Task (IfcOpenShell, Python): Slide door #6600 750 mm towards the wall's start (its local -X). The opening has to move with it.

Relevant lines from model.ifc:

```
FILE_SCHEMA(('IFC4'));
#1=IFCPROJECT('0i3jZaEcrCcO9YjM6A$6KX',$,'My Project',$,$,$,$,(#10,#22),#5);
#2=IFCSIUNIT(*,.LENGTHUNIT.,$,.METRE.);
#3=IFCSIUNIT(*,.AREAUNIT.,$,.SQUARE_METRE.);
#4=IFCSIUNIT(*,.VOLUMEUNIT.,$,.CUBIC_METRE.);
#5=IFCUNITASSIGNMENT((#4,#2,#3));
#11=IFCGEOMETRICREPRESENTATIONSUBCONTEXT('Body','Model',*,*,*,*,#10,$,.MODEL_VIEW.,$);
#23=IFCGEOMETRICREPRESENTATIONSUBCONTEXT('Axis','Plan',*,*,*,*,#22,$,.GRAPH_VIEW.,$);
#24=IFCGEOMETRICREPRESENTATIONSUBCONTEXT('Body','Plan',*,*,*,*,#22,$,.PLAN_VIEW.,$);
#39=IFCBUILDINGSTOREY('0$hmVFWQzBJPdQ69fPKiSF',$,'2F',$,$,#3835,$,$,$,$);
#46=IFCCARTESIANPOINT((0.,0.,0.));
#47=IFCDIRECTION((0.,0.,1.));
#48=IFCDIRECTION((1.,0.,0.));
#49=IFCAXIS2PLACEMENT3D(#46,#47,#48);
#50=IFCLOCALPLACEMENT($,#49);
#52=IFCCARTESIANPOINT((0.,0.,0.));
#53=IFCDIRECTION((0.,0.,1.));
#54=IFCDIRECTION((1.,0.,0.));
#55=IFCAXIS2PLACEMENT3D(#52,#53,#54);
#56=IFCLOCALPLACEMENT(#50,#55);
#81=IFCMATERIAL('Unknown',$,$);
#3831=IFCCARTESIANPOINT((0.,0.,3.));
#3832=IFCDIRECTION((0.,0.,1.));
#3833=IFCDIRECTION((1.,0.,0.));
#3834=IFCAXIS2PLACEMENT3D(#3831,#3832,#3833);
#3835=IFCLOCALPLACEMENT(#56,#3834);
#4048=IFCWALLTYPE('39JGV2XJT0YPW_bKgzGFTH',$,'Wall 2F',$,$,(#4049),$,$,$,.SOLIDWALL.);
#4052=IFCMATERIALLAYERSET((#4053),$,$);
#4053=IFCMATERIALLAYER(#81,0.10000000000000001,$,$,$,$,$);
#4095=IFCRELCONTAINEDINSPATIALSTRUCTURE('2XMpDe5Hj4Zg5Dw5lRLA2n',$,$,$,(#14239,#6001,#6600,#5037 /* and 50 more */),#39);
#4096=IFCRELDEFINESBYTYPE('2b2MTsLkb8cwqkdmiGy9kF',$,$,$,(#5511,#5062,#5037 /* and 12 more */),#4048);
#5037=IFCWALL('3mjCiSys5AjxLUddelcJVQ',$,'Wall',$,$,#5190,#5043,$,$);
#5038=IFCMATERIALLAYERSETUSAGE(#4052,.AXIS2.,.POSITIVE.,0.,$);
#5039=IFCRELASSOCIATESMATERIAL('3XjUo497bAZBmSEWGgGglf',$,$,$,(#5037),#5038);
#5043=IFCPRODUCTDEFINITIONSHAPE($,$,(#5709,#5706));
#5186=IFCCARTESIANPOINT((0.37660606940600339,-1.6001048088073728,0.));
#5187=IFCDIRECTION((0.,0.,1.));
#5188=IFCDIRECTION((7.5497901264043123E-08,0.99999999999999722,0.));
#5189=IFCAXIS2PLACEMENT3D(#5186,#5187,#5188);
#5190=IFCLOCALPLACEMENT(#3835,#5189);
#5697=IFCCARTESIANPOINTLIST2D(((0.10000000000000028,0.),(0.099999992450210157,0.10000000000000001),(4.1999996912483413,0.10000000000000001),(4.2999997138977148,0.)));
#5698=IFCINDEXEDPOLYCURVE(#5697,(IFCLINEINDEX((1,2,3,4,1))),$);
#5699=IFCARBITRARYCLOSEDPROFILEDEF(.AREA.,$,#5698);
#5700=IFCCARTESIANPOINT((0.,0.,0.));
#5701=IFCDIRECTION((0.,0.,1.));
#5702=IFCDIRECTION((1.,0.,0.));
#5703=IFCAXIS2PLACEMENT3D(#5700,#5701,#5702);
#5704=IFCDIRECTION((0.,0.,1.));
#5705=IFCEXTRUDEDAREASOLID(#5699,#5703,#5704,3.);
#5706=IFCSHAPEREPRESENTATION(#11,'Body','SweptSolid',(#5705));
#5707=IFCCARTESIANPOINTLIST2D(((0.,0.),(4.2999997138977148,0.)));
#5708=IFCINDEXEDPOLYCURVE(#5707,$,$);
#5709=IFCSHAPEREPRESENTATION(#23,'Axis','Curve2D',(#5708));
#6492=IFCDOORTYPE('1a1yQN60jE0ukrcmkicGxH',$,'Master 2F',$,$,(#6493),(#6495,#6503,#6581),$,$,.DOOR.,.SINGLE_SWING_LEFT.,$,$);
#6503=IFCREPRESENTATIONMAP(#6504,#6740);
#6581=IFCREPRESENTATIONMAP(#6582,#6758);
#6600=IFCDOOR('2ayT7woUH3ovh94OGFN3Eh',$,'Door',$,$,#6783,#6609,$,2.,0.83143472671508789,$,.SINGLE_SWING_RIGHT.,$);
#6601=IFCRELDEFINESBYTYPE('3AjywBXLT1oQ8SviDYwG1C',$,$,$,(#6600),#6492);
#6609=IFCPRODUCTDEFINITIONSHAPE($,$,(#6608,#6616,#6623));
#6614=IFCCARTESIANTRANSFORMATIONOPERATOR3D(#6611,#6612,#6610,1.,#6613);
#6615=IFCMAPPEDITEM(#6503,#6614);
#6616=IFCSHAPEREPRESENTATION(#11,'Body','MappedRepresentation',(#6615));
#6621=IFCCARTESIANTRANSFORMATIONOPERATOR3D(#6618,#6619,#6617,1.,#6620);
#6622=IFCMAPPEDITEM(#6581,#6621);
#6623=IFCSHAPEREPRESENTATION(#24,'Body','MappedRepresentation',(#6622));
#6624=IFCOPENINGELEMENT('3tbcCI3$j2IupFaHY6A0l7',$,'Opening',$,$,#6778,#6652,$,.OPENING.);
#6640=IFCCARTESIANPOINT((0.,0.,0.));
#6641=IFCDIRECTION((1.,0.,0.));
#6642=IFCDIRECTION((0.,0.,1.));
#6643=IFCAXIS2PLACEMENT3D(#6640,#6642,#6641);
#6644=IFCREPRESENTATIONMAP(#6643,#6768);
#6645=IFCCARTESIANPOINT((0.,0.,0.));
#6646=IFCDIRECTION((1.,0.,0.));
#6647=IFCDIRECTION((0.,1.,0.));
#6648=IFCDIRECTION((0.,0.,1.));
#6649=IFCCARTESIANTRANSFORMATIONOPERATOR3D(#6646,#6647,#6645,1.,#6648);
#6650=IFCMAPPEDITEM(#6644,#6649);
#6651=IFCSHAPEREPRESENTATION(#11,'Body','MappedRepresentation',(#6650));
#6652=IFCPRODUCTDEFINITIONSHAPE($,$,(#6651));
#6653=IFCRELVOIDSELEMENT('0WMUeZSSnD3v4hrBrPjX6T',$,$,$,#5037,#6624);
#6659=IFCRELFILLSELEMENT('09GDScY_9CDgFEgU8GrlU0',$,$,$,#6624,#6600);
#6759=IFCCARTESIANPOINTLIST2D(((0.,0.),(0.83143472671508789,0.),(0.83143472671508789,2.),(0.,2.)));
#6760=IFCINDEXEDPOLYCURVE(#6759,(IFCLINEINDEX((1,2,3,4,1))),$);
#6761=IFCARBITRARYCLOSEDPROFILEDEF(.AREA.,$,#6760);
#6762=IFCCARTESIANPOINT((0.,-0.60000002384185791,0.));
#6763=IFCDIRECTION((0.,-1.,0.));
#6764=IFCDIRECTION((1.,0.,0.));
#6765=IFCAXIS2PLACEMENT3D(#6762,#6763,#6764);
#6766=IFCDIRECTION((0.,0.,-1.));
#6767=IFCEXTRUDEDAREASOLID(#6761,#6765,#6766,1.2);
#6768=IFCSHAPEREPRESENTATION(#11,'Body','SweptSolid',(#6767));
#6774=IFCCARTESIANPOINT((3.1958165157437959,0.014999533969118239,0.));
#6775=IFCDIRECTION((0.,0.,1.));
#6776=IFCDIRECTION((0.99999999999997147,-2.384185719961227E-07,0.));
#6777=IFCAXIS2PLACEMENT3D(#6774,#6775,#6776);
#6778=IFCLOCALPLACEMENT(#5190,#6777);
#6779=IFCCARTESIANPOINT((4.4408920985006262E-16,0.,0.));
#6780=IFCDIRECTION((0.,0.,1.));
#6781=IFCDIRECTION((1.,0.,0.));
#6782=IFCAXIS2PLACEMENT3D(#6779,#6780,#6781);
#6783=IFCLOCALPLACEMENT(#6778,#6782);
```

```python
import ifcopenshell
import ifcopenshell.api.geometry
import ifcopenshell.util.placement

model = ifcopenshell.open("model.ifc")

door = model.by_guid("2ayT7woUH3ovh94OGFN3Eh")
opening = door.FillsVoids[0].RelatingOpeningElement
wall = opening.VoidsElements[0].RelatingBuildingElement

wall_matrix = ifcopenshell.util.placement.get_local_placement(wall.ObjectPlacement)
shift = wall_matrix[:3, 0] * -0.75
before = ifcopenshell.util.placement.get_local_placement(door.ObjectPlacement)[:3, 3].copy()

# The door is placed relative to its opening, so it follows when the opening moves.
matrix = ifcopenshell.util.placement.get_local_placement(opening.ObjectPlacement)
matrix[:3, 3] += shift
ifcopenshell.api.geometry.edit_object_placement(
    model, product=opening, matrix=matrix, is_si=False, should_transform_children=True
)

after = ifcopenshell.util.placement.get_local_placement(door.ObjectPlacement)[:3, 3]
print("door moved by", (after - before).round(3) + 0.0)

model.write("model_updated.ifc")
```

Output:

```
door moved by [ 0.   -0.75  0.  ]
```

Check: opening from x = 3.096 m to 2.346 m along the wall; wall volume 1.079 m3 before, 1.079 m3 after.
